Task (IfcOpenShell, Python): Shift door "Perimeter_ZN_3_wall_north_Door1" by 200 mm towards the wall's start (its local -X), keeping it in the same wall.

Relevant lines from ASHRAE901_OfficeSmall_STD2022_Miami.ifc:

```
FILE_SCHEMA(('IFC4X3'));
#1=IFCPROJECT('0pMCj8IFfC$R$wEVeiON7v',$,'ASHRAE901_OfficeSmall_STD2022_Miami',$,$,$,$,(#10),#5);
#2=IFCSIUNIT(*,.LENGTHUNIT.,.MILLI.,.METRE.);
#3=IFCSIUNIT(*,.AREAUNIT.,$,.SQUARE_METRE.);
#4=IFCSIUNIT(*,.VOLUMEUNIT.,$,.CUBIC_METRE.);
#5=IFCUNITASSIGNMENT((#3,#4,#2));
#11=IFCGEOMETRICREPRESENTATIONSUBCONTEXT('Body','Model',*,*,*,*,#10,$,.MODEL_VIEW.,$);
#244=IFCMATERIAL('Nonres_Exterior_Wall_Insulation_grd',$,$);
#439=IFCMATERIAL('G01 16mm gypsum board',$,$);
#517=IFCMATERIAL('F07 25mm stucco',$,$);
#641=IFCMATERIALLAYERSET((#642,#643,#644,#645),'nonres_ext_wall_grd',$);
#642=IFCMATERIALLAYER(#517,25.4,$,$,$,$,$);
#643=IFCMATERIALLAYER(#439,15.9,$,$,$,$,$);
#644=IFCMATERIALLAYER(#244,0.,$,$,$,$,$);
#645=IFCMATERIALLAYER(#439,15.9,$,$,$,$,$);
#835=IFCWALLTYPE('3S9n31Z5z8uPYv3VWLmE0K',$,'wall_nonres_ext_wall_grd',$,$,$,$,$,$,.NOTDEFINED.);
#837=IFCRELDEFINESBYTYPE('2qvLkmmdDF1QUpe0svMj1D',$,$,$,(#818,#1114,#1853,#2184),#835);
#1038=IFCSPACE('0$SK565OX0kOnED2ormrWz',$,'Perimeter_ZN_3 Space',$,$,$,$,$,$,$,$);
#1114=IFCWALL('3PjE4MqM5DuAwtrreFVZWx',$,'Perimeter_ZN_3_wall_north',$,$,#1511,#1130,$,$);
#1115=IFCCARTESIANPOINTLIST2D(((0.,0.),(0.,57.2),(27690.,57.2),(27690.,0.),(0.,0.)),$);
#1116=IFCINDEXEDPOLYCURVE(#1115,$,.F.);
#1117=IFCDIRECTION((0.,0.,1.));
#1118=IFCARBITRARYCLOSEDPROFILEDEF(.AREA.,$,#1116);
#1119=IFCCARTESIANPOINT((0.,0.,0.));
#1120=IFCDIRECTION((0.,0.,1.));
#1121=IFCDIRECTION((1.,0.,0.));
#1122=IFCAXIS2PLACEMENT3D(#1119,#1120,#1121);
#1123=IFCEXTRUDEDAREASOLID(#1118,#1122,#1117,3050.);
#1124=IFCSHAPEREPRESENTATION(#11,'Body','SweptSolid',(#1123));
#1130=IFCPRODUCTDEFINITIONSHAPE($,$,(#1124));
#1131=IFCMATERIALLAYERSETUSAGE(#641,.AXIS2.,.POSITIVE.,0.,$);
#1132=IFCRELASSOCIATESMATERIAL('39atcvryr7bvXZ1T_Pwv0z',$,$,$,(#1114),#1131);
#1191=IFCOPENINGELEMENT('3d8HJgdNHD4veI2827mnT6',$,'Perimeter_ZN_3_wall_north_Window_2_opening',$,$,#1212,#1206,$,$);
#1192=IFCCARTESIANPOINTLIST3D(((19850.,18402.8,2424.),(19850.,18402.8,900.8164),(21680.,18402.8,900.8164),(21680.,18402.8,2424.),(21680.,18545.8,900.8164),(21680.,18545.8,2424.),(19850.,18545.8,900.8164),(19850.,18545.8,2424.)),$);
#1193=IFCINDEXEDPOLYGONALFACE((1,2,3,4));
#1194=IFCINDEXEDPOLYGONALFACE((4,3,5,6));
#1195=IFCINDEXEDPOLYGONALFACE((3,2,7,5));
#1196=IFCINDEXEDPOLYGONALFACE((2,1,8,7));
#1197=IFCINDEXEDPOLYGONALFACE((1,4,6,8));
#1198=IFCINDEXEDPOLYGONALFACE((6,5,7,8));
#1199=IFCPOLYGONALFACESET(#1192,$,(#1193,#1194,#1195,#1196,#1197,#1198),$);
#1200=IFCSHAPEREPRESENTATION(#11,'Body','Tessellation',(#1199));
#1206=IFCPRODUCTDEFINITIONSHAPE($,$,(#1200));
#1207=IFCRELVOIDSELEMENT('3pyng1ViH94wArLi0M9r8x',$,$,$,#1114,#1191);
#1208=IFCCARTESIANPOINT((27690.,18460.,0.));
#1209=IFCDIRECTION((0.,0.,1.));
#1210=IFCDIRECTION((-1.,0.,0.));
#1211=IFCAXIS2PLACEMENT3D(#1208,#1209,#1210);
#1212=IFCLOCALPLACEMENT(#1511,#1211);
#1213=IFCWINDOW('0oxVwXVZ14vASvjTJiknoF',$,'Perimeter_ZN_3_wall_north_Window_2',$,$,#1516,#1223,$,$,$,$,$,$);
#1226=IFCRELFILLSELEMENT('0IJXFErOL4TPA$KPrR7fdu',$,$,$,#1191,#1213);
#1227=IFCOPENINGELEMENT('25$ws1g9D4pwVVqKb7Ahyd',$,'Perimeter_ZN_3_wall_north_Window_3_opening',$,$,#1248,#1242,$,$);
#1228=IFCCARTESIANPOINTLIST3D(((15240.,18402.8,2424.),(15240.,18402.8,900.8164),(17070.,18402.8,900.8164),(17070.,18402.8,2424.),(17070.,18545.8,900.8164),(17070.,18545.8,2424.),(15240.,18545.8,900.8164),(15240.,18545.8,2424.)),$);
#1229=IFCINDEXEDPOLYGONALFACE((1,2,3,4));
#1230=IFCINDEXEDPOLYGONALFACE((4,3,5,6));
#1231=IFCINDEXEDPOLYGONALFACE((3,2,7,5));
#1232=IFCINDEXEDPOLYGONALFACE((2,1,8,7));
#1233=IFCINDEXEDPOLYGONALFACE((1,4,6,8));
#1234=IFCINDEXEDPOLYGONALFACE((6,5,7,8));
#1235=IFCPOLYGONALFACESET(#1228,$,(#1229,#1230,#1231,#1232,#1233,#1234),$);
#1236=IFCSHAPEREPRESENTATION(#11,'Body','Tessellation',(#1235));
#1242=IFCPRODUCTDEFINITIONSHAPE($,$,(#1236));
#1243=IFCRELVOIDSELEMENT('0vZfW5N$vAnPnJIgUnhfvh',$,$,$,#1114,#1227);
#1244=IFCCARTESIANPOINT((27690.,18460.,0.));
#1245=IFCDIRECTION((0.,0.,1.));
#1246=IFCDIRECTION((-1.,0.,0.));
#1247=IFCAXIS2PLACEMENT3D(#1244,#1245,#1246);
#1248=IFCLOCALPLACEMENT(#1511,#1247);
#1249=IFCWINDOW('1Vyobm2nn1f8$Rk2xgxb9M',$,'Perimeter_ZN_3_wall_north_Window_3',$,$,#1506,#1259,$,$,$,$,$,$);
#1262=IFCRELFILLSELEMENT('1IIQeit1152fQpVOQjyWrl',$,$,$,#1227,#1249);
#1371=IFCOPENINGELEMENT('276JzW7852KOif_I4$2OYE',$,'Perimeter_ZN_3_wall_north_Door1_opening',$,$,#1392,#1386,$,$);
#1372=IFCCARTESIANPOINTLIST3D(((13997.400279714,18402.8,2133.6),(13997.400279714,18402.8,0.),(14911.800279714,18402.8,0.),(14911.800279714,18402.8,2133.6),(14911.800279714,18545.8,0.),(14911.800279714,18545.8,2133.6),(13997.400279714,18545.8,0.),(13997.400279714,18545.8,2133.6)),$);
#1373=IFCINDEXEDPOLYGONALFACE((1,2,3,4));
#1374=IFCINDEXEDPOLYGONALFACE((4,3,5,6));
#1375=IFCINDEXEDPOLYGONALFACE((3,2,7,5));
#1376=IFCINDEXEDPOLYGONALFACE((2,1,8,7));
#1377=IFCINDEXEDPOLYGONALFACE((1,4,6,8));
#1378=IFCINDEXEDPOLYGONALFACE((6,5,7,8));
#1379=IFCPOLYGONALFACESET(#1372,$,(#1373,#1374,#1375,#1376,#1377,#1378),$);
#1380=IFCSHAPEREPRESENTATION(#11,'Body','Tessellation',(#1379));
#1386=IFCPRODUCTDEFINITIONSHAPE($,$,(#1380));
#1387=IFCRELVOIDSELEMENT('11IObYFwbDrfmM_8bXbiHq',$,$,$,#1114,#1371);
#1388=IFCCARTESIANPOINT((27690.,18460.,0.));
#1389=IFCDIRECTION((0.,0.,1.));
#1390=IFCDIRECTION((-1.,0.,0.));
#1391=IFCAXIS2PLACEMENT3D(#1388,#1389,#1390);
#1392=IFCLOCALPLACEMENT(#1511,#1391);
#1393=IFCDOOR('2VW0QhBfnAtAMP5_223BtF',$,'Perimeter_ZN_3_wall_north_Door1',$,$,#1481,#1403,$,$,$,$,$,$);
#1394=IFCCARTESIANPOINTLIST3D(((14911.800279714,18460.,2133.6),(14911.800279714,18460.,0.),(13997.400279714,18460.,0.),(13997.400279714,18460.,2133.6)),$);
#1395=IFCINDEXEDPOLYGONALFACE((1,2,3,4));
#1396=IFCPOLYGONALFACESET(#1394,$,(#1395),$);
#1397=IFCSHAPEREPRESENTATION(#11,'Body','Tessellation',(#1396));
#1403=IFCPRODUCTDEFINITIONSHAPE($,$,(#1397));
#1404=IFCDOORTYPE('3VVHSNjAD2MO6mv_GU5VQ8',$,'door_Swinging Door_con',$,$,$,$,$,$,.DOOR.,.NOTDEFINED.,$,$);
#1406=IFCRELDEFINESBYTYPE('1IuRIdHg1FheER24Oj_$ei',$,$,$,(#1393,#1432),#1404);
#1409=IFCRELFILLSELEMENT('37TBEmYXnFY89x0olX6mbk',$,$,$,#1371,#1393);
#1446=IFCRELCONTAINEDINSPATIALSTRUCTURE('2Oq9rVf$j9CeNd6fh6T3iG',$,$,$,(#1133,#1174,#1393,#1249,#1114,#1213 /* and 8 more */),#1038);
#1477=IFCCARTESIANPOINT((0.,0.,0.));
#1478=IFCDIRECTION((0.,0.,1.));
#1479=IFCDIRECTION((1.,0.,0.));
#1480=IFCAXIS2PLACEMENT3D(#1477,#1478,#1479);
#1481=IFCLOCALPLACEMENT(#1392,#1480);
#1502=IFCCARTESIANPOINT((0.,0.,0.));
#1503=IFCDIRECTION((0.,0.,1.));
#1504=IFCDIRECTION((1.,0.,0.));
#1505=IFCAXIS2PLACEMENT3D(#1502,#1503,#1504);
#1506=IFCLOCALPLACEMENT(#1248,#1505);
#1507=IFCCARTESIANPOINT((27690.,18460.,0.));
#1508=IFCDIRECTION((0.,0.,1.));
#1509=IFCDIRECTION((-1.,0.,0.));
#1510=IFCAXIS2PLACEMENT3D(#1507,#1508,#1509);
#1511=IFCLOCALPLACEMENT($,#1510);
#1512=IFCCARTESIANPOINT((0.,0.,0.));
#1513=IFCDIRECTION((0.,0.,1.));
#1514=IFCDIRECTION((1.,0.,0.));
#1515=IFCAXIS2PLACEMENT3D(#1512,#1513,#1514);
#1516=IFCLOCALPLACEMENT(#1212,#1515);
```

```python
import ifcopenshell
import ifcopenshell.api.geometry
import ifcopenshell.util.placement
import ifcopenshell.util.unit

model = ifcopenshell.open("ASHRAE901_OfficeSmall_STD2022_Miami.ifc")
unit_scale = ifcopenshell.util.unit.calculate_unit_scale(model)

door = model.by_id(1393)
opening = door.FillsVoids[0].RelatingOpeningElement
wall = opening.VoidsElements[0].RelatingBuildingElement

wall_matrix = ifcopenshell.util.placement.get_local_placement(wall.ObjectPlacement)
shift = wall_matrix[:3, 0] * -0.2 / unit_scale
before = ifcopenshell.util.placement.get_local_placement(door.ObjectPlacement)[:3, 3].copy()

# The door is placed relative to its opening, so it follows when the opening moves.
matrix = ifcopenshell.util.placement.get_local_placement(opening.ObjectPlacement)
matrix[:3, 3] += shift
ifcopenshell.api.geometry.edit_object_placement(
    model, product=opening, matrix=matrix, is_si=False, should_transform_children=True
)

after = ifcopenshell.util.placement.get_local_placement(door.ObjectPlacement)[:3, 3]
print("door moved by", (after - before).round(3) + 0.0)

model.write("ASHRAE901_OfficeSmall_STD2022_Miami_edited.ifc")
```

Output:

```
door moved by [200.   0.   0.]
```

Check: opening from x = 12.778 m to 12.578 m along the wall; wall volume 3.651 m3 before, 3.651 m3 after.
